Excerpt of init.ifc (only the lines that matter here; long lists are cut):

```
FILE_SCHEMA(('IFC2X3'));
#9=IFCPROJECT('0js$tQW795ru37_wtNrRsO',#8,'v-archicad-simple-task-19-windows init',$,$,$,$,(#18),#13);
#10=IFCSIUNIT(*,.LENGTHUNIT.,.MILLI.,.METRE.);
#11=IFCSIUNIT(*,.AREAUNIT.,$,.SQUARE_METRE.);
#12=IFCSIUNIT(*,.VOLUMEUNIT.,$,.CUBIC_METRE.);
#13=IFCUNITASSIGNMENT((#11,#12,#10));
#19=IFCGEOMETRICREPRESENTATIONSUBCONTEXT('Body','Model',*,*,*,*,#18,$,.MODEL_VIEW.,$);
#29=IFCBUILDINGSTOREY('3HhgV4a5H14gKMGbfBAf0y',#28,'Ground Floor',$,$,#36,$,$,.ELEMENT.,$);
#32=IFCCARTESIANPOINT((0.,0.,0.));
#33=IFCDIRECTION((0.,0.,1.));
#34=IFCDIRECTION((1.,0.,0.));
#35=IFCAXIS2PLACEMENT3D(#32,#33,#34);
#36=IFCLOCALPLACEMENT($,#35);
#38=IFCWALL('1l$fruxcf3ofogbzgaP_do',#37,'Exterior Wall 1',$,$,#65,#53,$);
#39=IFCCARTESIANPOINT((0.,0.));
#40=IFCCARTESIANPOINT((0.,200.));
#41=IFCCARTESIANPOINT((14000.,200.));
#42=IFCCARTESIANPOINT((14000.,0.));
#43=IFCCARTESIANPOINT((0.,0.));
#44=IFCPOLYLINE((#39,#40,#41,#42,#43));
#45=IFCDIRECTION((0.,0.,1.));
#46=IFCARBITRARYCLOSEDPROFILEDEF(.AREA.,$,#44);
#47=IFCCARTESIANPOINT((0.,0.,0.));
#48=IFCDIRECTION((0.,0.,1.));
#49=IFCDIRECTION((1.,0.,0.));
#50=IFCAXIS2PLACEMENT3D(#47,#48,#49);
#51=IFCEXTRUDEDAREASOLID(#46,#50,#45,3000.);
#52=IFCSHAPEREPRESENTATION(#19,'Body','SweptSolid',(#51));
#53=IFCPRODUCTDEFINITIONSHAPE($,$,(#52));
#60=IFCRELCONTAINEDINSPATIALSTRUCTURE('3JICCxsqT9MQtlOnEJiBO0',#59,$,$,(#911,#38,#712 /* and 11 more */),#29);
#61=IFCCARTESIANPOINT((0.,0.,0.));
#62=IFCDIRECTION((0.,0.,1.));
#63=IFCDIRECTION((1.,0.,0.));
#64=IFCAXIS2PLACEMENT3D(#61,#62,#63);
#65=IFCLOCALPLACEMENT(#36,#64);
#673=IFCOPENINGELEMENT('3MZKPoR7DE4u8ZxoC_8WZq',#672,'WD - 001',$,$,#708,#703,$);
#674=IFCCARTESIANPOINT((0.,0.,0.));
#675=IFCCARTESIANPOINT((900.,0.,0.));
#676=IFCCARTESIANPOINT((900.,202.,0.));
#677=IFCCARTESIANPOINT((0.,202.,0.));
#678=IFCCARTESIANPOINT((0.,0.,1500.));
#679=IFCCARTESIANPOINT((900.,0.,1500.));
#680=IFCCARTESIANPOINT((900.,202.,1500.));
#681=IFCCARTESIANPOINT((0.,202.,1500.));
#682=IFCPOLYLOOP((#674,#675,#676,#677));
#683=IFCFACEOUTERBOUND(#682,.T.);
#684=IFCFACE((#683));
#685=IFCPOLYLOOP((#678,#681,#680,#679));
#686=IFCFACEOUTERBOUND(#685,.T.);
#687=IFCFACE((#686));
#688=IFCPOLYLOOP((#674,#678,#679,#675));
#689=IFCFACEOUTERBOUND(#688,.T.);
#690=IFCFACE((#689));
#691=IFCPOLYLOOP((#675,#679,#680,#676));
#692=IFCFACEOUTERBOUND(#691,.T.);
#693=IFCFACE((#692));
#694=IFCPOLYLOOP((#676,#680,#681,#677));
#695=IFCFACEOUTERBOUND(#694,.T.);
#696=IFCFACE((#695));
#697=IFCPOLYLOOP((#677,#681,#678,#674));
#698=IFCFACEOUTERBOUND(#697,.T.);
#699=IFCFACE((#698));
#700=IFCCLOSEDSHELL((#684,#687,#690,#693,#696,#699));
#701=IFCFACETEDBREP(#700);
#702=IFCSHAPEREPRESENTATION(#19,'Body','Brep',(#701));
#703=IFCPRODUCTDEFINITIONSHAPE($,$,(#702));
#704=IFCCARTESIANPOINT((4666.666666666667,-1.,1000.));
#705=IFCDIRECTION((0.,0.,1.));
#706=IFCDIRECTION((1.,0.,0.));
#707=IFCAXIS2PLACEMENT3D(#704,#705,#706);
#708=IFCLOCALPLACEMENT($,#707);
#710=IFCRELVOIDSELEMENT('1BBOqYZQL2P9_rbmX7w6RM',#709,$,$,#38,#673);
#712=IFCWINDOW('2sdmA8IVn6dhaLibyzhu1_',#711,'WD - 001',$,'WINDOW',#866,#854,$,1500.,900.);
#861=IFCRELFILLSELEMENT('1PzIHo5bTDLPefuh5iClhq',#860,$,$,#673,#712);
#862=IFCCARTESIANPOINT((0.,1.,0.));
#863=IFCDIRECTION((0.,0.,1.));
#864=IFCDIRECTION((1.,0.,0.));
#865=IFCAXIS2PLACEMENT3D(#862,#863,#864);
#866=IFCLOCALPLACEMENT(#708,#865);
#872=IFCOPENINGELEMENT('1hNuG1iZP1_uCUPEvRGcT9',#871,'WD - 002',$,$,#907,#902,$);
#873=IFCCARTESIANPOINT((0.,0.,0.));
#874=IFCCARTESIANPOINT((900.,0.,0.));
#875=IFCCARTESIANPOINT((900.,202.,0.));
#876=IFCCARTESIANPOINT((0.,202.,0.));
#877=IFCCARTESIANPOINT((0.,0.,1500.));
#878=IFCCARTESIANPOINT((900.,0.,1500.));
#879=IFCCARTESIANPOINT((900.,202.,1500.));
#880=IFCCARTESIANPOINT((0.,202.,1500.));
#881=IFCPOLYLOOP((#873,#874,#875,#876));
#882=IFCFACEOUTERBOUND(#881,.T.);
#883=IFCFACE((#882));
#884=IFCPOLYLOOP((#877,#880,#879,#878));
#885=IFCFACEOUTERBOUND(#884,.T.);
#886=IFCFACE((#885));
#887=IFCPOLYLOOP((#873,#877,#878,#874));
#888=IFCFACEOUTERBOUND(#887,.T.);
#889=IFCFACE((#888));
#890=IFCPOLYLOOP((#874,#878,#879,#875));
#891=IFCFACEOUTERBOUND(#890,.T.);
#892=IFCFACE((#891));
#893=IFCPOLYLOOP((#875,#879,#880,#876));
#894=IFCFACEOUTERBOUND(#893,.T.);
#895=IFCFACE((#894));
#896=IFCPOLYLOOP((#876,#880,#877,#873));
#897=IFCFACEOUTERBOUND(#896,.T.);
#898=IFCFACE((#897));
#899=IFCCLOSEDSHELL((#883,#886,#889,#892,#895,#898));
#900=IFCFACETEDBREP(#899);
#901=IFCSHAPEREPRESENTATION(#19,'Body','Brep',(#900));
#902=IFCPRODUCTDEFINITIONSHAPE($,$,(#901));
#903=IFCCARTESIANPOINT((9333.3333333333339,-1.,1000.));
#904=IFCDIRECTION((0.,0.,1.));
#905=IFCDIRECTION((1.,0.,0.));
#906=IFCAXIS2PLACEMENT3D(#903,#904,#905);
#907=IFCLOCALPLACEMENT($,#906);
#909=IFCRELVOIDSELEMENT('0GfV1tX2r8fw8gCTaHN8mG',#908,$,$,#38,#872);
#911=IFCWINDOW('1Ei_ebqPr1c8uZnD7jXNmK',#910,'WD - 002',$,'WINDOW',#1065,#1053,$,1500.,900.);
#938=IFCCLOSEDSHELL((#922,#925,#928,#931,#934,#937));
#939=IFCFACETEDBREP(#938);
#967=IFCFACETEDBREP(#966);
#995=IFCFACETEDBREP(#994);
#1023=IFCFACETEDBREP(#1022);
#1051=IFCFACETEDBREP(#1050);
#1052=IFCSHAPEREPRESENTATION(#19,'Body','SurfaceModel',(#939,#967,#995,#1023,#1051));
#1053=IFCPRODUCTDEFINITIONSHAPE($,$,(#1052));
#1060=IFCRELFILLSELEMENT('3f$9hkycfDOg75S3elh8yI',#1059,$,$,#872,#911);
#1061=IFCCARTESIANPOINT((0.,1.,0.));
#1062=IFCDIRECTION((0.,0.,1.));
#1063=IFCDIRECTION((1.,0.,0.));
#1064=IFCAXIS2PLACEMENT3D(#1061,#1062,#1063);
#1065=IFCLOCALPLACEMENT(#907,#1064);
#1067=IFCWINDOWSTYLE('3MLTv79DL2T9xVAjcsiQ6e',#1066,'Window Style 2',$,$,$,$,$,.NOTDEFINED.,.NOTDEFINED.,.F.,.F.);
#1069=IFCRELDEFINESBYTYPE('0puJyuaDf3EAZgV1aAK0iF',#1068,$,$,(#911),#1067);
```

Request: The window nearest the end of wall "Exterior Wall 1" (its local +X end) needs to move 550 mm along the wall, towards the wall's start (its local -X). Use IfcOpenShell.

```python
import ifcopenshell
import ifcopenshell.api.geometry
import ifcopenshell.util.placement
import ifcopenshell.util.unit

model = ifcopenshell.open("init.ifc")
unit_scale = ifcopenshell.util.unit.calculate_unit_scale(model)

window = model.by_guid("1Ei_ebqPr1c8uZnD7jXNmK")
opening = window.FillsVoids[0].RelatingOpeningElement
wall = opening.VoidsElements[0].RelatingBuildingElement

wall_matrix = ifcopenshell.util.placement.get_local_placement(wall.ObjectPlacement)
shift = wall_matrix[:3, 0] * -0.55 / unit_scale
before = ifcopenshell.util.placement.get_local_placement(window.ObjectPlacement)[:3, 3].copy()

# The window is placed relative to its opening, so it follows when the opening moves.
matrix = ifcopenshell.util.placement.get_local_placement(opening.ObjectPlacement)
matrix[:3, 3] += shift
ifcopenshell.api.geometry.edit_object_placement(
    model, product=opening, matrix=matrix, is_si=False, should_transform_children=True
)

after = ifcopenshell.util.placement.get_local_placement(window.ObjectPlacement)[:3, 3]
print("window moved by", (after - before).round(3) + 0.0)

model.write("init-out.ifc")
```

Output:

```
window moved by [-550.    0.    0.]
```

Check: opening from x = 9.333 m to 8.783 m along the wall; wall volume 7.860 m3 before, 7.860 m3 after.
